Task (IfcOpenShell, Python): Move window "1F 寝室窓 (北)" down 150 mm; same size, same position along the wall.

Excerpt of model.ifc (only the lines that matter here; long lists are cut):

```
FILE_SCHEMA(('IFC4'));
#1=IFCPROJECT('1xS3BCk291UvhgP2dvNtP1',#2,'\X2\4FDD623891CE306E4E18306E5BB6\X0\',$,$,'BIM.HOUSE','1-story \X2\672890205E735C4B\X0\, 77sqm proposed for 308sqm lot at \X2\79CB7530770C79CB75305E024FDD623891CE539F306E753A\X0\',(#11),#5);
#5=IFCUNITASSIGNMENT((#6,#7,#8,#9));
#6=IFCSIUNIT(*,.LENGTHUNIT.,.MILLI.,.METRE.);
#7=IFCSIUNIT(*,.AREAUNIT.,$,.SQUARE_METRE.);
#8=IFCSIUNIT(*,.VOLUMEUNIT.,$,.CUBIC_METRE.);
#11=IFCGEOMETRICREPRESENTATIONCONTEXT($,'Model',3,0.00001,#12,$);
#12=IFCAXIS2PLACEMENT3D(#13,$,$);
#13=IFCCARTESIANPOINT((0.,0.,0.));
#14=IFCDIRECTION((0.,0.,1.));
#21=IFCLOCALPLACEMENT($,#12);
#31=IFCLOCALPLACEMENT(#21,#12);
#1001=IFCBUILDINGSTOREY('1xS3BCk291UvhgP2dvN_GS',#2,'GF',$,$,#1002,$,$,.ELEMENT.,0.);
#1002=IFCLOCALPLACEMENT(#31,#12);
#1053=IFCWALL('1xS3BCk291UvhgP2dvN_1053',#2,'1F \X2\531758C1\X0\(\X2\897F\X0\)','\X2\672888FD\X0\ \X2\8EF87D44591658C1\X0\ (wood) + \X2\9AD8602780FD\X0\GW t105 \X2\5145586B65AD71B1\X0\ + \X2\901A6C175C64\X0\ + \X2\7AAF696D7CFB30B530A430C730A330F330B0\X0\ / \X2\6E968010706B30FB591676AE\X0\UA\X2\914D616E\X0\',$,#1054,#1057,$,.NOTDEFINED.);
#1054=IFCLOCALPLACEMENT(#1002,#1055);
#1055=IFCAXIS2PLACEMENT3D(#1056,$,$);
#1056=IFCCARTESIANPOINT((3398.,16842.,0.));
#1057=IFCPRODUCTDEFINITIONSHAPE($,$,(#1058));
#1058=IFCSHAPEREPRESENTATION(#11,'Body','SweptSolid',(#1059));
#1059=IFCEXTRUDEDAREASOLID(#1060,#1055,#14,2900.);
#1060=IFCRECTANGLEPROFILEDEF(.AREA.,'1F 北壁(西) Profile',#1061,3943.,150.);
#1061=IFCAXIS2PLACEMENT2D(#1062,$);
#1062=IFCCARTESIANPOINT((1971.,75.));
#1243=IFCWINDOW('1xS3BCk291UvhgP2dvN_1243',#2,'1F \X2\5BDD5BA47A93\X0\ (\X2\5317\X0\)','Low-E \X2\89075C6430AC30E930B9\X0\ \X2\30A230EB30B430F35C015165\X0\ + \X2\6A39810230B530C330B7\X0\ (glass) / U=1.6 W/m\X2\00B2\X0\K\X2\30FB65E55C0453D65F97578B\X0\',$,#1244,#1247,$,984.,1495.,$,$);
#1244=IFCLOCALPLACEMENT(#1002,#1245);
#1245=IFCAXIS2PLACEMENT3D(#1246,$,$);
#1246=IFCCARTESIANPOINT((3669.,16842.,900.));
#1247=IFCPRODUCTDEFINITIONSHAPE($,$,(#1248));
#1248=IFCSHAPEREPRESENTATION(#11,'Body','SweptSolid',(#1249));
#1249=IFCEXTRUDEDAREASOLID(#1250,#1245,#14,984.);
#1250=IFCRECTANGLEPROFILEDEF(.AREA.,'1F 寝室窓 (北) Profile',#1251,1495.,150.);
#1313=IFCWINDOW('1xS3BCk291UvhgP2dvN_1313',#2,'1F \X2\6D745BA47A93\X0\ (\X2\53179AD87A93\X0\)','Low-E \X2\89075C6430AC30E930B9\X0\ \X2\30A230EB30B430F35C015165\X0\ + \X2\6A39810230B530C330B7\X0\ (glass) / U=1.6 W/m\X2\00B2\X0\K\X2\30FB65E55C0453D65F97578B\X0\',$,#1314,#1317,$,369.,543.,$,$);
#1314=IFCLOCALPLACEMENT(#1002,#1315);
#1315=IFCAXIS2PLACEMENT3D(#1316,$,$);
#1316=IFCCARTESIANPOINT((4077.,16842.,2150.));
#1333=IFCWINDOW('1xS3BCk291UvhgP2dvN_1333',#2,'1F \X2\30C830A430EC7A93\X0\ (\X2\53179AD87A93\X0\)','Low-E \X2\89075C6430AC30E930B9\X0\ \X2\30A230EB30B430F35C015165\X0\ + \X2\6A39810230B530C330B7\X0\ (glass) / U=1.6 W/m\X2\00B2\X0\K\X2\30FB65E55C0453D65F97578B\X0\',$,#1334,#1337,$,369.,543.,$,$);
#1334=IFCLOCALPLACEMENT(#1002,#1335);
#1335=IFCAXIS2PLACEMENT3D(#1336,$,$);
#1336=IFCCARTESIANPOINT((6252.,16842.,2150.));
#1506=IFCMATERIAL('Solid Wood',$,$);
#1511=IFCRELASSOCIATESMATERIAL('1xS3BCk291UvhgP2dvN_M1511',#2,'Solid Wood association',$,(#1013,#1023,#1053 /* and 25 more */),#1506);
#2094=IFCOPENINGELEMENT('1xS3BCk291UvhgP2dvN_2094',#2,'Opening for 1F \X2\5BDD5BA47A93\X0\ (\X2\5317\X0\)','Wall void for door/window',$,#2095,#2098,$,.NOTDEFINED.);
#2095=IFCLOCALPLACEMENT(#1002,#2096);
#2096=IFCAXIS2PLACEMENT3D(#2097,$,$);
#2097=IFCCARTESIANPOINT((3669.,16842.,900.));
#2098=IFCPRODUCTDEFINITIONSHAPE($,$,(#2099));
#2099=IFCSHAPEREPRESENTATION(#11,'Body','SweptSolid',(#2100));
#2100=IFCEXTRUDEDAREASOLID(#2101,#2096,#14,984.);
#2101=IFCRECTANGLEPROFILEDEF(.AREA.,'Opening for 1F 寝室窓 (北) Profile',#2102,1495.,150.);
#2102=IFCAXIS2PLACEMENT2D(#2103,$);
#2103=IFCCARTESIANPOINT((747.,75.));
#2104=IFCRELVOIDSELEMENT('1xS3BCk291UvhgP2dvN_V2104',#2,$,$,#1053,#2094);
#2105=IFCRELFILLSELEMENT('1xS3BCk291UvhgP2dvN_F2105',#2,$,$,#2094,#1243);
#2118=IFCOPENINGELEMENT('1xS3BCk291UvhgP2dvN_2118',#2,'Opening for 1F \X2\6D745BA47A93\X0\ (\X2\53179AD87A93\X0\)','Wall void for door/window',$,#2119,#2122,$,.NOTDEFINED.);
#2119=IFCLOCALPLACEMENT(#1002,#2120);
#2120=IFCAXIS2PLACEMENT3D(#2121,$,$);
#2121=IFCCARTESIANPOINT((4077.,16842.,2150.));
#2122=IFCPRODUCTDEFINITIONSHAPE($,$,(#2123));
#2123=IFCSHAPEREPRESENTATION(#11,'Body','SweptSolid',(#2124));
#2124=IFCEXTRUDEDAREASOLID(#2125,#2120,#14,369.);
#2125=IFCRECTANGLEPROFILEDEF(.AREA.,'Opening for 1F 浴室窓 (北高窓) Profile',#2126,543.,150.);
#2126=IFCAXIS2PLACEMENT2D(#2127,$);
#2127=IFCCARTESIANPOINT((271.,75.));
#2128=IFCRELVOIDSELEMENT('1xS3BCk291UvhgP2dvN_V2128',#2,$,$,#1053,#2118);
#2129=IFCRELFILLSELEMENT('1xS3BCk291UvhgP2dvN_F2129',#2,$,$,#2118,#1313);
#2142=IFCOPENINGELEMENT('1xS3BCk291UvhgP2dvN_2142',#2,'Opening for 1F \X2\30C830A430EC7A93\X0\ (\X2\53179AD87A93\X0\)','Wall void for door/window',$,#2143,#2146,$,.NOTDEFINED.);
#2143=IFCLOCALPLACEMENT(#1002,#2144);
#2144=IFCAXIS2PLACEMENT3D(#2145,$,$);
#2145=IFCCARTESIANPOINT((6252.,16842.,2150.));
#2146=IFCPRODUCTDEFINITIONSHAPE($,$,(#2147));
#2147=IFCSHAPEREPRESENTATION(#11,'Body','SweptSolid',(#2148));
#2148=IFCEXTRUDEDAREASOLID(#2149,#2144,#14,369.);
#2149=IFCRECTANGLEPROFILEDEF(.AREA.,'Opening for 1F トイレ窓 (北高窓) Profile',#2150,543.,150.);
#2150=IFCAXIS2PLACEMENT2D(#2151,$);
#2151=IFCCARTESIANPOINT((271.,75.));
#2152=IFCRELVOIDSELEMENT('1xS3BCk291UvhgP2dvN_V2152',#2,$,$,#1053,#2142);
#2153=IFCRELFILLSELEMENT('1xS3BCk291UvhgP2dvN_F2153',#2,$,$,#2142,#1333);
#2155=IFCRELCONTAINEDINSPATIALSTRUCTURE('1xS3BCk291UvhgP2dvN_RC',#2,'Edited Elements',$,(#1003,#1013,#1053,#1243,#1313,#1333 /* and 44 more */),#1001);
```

```python
import numpy as np
import ifcopenshell
import ifcopenshell.api.geometry
import ifcopenshell.util.placement
import ifcopenshell.util.unit

model = ifcopenshell.open("model.ifc")
unit_scale = ifcopenshell.util.unit.calculate_unit_scale(model)

window = model.by_id(1243)
opening = window.FillsVoids[0].RelatingOpeningElement
dz = -0.15 / unit_scale

shift = np.array([0.0, 0.0, dz])
# The window is not placed relative to its opening, so move both.
for product in (opening, window):
    matrix = ifcopenshell.util.placement.get_local_placement(product.ObjectPlacement)
    matrix[:3, 3] += shift
    ifcopenshell.api.geometry.edit_object_placement(model, product=product, matrix=matrix, is_si=False)

print(f"moved by {dz * unit_scale:+.3f} m")

model.write("model_edited.ifc")
```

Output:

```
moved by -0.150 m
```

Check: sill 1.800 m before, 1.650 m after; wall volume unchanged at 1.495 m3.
